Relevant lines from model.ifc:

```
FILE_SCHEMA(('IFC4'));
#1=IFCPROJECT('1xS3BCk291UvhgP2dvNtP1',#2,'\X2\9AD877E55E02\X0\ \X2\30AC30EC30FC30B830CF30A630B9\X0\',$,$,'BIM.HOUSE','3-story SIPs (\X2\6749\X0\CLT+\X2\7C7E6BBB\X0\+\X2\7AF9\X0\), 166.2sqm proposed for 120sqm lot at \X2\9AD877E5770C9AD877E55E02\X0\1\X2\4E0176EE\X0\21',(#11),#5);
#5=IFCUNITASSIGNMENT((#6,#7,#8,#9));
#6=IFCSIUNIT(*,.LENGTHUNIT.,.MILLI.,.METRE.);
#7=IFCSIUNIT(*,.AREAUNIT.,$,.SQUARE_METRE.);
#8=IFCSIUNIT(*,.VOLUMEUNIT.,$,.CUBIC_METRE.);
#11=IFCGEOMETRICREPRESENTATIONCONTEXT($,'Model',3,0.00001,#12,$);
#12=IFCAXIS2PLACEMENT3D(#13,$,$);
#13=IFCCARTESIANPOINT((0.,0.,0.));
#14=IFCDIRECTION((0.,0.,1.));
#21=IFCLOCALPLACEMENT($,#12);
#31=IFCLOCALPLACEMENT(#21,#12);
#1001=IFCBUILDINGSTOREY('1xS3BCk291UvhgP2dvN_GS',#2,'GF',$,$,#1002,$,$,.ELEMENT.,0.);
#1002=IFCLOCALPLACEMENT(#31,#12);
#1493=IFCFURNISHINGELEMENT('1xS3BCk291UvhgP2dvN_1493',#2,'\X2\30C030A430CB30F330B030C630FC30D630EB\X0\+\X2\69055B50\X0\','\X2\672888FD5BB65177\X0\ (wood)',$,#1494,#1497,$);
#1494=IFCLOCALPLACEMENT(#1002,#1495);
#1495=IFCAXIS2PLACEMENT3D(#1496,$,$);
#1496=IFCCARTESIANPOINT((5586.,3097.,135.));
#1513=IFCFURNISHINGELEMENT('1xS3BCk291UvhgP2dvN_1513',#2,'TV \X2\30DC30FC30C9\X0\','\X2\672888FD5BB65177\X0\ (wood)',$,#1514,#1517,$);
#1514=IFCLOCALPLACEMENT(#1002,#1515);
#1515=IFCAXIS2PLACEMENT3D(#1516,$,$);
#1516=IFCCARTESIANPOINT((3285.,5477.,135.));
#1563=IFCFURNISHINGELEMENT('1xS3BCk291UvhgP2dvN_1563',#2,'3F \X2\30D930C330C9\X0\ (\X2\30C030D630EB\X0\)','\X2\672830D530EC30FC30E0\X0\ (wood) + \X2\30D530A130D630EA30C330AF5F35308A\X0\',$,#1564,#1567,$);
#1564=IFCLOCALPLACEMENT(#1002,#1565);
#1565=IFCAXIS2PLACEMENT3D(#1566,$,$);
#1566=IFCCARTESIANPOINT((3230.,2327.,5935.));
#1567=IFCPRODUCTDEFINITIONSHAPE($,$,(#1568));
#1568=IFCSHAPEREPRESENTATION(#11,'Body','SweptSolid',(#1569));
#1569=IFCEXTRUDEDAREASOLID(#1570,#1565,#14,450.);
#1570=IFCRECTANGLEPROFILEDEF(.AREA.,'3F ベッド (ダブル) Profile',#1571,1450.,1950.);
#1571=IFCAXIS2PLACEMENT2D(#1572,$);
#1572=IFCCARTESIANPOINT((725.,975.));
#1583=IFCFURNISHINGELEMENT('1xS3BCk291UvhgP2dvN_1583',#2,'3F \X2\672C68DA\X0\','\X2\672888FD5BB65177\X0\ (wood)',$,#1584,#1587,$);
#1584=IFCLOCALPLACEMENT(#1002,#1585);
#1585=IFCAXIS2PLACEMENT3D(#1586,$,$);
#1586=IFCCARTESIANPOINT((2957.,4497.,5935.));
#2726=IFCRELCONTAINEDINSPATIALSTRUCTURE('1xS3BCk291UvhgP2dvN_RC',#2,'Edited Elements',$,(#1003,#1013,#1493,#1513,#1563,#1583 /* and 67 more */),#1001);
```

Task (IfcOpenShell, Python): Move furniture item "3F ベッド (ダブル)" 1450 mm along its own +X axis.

```python
import ifcopenshell
import ifcopenshell.api.geometry
import ifcopenshell.util.placement
import ifcopenshell.util.unit

model = ifcopenshell.open("model.ifc")
unit_scale = ifcopenshell.util.unit.calculate_unit_scale(model)

item = model.by_guid("1xS3BCk291UvhgP2dvN_1563")
matrix = ifcopenshell.util.placement.get_local_placement(item.ObjectPlacement)
matrix[:3, 3] += matrix[:3, 0] * 1.45 / unit_scale
ifcopenshell.api.geometry.edit_object_placement(model, product=item, matrix=matrix, is_si=False)

print(ifcopenshell.util.placement.get_local_placement(item.ObjectPlacement).round(3) + 0.0)

model.write("model-out.ifc")
```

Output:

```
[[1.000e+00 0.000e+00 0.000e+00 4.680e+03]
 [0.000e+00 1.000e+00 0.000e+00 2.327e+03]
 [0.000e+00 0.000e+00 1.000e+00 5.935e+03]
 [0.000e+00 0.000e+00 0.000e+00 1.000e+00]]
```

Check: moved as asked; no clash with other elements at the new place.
